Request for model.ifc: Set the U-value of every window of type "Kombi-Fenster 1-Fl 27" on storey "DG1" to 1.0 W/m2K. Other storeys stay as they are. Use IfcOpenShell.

First a look at what the model holds.

```python
import ifcopenshell
import ifcopenshell.util.element

model = ifcopenshell.open("model.ifc")
print(model.schema)
storey = next(s for s in model.by_type("IfcBuildingStorey") if s.Name == "DG1")
windows = [e for e in ifcopenshell.util.element.get_decomposition(storey) if e.is_a("IfcWindow")]
seen = {}
for e in windows:
    element_type = ifcopenshell.util.element.get_type(e)
    key = (element_type.Name if element_type != e and element_type else None, ifcopenshell.util.element.get_pset(e, "Pset_WindowCommon", "ThermalTransmittance"))
    seen[key] = seen.get(key, 0) + 1
for (name, value), count in sorted(seen.items(), key=str):
    print(count, "x", name, "|", value)
```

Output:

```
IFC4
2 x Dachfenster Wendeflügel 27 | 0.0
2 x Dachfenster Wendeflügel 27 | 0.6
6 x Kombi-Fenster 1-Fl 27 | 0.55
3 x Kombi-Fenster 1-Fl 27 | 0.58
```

```python
import ifcopenshell
import ifcopenshell.api.pset
import ifcopenshell.util.element

model = ifcopenshell.open("model.ifc")

storey = next(s for s in model.by_type("IfcBuildingStorey") if s.Name == "DG1")
windows = [e for e in ifcopenshell.util.element.get_decomposition(storey) if e.is_a("IfcWindow")]

count = 0
for e in windows:
    element_type = ifcopenshell.util.element.get_type(e)
    if element_type in (None, e) or element_type.Name != "Kombi-Fenster 1-Fl 27":
        continue
    # add_pset returns the element's existing set when there is one.
    pset = ifcopenshell.api.pset.add_pset(model, product=e, name="Pset_WindowCommon")
    ifcopenshell.api.pset.edit_pset(model, pset=pset, properties={"ThermalTransmittance": 1.0})
    count += 1

print(count, "windows updated")

model.write("model_edited.ifc")
```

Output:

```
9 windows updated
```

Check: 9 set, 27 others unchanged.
